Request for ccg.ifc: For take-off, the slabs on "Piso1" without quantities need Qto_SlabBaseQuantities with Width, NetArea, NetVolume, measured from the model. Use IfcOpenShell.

First a look at what the model holds.

```python
import ifcopenshell
import ifcopenshell.util.element
import ifcopenshell.util.unit

model = ifcopenshell.open("ccg.ifc")
print(model.schema)
for unit_type in ("LENGTHUNIT", "AREAUNIT", "VOLUMEUNIT"):
    print(unit_type, ifcopenshell.util.unit.calculate_unit_scale(model, unit_type))
storey = next(s for s in model.by_type("IfcBuildingStorey") if s.Name == "Piso1")
slabs = [e for e in ifcopenshell.util.element.get_decomposition(storey) if e.is_a("IfcSlab")]
for e in sorted(slabs, key=lambda e: e.id()):
    print(e.id(), e.is_a(), e.Name, list(ifcopenshell.util.element.get_psets(e, qtos_only=True)), sep=" | ")
```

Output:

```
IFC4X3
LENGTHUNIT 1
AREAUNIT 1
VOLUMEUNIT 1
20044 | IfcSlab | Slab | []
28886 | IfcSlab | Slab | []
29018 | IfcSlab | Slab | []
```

```python
import ifcopenshell
import ifcopenshell.api.pset
import ifcopenshell.geom
import ifcopenshell.util.element
import ifcopenshell.util.shape
import ifcopenshell.util.unit

model = ifcopenshell.open("ccg.ifc")
unit_scale = ifcopenshell.util.unit.calculate_unit_scale(model)
area_scale = ifcopenshell.util.unit.calculate_unit_scale(model, "AREAUNIT")
volume_scale = ifcopenshell.util.unit.calculate_unit_scale(model, "VOLUMEUNIT")
settings = ifcopenshell.geom.settings()

storey = next(s for s in model.by_type("IfcBuildingStorey") if s.Name == "Piso1")
slabs = [e for e in ifcopenshell.util.element.get_decomposition(storey) if e.is_a("IfcSlab")]

for e in sorted(slabs, key=lambda e: e.id()):
    if ifcopenshell.util.element.get_psets(e, qtos_only=True, should_inherit=False):
        continue
    # Geometry comes back in metres, in the element's own axes.
    shape = ifcopenshell.geom.create_shape(settings, e)
    values = {
        "Width": ifcopenshell.util.shape.get_z(shape.geometry) / unit_scale,
        "NetArea": ifcopenshell.util.shape.get_footprint_area(shape.geometry) / area_scale,
        "NetVolume": ifcopenshell.util.shape.get_volume(shape.geometry) / volume_scale,
    }
    qto = ifcopenshell.api.pset.add_qto(model, product=e, name="Qto_SlabBaseQuantities")
    ifcopenshell.api.pset.edit_qto(model, qto=qto, properties=values)
    print(e.id(), {k: round(v, 3) for k, v in values.items()})

model.write("ccg-out.ifc")
```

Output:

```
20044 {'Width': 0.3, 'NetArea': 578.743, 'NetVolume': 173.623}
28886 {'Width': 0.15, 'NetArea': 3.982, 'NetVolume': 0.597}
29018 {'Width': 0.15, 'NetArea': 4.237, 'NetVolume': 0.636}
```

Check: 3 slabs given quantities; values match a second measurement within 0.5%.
